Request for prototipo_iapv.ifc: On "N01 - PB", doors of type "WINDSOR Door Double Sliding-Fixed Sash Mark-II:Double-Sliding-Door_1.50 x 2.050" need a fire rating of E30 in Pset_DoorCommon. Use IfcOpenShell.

First a look at what the model holds.

```python
import ifcopenshell
import ifcopenshell.util.element

model = ifcopenshell.open("prototipo_iapv.ifc")
print(model.schema)
storey = next(s for s in model.by_type("IfcBuildingStorey") if s.Name == "N01 - PB")
doors = [e for e in ifcopenshell.util.element.get_decomposition(storey) if e.is_a("IfcDoor")]
seen = {}
for e in doors:
    element_type = ifcopenshell.util.element.get_type(e)
    key = (element_type.Name if element_type != e and element_type else None, ifcopenshell.util.element.get_pset(e, "Pset_DoorCommon", "FireRating"))
    seen[key] = seen.get(key, 0) + 1
for (name, value), count in sorted(seen.items(), key=str):
    print(count, "x", name, "|", value)
```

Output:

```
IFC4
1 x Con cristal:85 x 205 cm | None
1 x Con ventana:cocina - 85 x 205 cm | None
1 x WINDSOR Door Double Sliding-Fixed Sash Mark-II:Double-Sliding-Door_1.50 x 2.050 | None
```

```python
import ifcopenshell
import ifcopenshell.api.pset
import ifcopenshell.util.element

model = ifcopenshell.open("prototipo_iapv.ifc")

storey = next(s for s in model.by_type("IfcBuildingStorey") if s.Name == "N01 - PB")
doors = [e for e in ifcopenshell.util.element.get_decomposition(storey) if e.is_a("IfcDoor")]

count = 0
for e in doors:
    element_type = ifcopenshell.util.element.get_type(e)
    if element_type in (None, e) or element_type.Name != "WINDSOR Door Double Sliding-Fixed Sash Mark-II:Double-Sliding-Door_1.50 x 2.050":
        continue
    # add_pset returns the element's existing set when there is one.
    pset = ifcopenshell.api.pset.add_pset(model, product=e, name="Pset_DoorCommon")
    ifcopenshell.api.pset.edit_pset(model, pset=pset, properties={"FireRating": "E30"})
    count += 1

print(count, "doors updated")

model.write("prototipo_iapv-out.ifc")
```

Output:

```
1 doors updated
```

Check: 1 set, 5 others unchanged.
